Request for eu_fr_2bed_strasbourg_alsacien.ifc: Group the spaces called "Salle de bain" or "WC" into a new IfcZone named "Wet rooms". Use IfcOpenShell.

First a look at what the model holds.

```python
import ifcopenshell

model = ifcopenshell.open("eu_fr_2bed_strasbourg_alsacien.ifc")
print(model.schema)
seen = {}
for space in model.by_type("IfcSpace"):
    seen[space.LongName] = seen.get(space.LongName, 0) + 1
for name, count in sorted(seen.items(), key=str):
    print(count, "x", name)
print("zones:", [z.Name for z in model.by_type("IfcZone")][:20])
```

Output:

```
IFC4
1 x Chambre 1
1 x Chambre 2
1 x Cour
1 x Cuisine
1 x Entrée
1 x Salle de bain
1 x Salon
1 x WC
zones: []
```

```python
import ifcopenshell
import ifcopenshell.api.group
import ifcopenshell.api.root

model = ifcopenshell.open("eu_fr_2bed_strasbourg_alsacien.ifc")

names = {"Salle de bain", "WC"}
spaces = [s for s in model.by_type("IfcSpace") if s.LongName in names]

zone = ifcopenshell.api.root.create_entity(model, ifc_class="IfcZone", name="Wet rooms")
ifcopenshell.api.group.assign_group(model, products=spaces, group=zone)
print(len(spaces), "spaces in", zone.Name)

model.write("eu_fr_2bed_strasbourg_alsacien_v2.ifc")
```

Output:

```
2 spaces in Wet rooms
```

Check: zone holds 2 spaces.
